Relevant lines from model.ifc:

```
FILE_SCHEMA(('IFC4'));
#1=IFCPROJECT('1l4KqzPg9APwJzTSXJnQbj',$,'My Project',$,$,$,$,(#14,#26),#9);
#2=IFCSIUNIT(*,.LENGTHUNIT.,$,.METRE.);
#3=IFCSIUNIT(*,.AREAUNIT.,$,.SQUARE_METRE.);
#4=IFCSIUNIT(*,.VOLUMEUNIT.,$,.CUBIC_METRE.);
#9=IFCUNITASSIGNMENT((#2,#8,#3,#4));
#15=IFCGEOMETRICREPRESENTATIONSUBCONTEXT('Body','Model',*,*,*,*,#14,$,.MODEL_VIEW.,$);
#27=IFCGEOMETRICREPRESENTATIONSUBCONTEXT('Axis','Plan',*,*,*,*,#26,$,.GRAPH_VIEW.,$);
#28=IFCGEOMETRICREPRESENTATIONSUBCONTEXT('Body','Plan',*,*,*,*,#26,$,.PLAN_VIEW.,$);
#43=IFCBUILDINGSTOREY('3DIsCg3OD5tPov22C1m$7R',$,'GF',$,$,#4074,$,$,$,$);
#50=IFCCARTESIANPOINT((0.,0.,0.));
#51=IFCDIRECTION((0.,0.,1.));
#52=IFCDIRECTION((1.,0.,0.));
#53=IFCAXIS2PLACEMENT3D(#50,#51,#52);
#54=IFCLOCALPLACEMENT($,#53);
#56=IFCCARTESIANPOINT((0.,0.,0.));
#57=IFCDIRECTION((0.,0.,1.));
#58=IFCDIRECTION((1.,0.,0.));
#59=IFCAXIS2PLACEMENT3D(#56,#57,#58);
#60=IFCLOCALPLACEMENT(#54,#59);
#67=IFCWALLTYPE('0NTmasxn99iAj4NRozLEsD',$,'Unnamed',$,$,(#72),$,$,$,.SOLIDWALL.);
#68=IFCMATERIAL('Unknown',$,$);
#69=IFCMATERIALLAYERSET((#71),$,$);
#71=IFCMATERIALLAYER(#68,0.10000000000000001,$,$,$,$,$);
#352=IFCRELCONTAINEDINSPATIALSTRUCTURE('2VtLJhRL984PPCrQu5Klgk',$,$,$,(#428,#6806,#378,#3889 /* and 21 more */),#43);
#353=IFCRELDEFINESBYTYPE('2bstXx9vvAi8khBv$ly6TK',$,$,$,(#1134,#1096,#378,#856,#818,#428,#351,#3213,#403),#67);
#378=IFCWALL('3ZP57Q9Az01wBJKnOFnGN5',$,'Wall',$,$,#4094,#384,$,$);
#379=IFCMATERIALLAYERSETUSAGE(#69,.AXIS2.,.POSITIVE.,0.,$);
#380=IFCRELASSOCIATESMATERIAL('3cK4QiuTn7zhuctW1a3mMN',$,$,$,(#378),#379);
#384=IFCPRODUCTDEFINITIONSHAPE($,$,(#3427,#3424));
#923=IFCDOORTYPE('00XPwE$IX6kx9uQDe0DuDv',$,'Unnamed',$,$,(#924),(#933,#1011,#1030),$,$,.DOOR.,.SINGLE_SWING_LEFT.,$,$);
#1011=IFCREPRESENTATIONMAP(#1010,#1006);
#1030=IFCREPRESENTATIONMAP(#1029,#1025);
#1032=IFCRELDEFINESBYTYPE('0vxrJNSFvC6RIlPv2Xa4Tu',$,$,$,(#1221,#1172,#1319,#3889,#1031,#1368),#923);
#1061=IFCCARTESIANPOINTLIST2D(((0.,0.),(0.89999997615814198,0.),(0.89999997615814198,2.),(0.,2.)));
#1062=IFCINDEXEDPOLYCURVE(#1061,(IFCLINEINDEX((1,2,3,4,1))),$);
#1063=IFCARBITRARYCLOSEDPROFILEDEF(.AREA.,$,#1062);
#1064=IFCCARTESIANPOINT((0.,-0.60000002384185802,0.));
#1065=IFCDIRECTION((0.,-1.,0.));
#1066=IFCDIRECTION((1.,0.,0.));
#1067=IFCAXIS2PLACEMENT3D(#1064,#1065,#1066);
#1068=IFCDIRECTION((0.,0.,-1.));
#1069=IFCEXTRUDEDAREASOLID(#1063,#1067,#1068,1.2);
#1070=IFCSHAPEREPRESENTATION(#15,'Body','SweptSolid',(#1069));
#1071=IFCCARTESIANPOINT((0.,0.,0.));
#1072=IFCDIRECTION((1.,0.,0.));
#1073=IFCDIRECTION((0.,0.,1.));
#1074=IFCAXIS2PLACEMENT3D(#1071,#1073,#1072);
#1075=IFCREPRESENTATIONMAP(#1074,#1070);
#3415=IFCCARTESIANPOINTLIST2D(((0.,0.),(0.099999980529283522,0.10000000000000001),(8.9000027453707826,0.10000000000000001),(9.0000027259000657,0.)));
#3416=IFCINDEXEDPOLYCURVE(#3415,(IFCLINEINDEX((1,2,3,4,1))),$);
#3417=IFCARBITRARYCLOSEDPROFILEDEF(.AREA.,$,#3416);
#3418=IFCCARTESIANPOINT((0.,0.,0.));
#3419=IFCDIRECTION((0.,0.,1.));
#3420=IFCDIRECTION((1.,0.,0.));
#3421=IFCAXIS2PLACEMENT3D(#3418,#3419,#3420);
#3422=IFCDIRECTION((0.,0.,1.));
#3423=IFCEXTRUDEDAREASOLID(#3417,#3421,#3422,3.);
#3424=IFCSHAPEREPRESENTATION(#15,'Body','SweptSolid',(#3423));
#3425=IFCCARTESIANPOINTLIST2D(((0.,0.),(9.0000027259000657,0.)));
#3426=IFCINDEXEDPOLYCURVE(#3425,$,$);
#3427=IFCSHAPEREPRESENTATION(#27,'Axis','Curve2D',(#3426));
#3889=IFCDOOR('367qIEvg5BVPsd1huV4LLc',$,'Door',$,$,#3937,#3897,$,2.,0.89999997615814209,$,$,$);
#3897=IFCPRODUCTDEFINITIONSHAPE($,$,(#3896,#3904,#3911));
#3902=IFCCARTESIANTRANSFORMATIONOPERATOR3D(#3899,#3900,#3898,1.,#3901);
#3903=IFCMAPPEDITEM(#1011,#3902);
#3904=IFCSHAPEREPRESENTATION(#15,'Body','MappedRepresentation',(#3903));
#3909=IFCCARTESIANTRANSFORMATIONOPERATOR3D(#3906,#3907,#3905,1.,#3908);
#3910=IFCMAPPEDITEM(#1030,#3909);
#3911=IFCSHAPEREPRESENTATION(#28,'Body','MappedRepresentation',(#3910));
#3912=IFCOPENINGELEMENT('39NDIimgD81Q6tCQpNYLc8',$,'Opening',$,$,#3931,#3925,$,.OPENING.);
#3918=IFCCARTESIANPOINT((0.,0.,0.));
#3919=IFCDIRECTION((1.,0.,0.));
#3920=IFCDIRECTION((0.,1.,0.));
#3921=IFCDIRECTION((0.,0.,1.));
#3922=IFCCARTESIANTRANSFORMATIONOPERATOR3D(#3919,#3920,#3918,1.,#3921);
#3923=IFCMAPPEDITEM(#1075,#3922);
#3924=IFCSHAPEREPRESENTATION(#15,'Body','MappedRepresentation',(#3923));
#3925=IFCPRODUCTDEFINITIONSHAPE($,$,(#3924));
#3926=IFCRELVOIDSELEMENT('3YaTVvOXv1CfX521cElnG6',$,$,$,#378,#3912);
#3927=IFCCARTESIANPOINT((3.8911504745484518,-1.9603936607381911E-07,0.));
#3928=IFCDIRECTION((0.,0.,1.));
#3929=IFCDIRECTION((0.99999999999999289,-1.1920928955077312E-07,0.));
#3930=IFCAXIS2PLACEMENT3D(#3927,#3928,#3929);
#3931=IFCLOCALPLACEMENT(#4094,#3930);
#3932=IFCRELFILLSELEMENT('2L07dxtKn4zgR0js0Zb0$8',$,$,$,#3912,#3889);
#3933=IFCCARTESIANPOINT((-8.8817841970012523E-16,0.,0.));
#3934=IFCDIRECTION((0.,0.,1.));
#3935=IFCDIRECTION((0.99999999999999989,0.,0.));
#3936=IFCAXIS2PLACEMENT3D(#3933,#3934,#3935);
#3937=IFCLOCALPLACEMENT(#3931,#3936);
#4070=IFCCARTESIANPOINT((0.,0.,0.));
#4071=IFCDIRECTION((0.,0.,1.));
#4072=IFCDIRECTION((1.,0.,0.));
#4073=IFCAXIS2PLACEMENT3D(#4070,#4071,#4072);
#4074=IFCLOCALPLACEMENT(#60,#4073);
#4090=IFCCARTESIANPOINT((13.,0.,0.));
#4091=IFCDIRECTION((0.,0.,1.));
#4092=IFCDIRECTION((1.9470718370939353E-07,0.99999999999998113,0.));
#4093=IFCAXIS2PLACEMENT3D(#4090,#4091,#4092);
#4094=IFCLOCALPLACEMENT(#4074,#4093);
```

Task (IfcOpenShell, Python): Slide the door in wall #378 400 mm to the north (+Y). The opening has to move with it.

```python
import ifcopenshell
import ifcopenshell.api.geometry
import ifcopenshell.util.placement
import ifcopenshell.util.unit

model = ifcopenshell.open("model.ifc")
unit_scale = ifcopenshell.util.unit.calculate_unit_scale(model)

door = model.by_guid("367qIEvg5BVPsd1huV4LLc")
opening = door.FillsVoids[0].RelatingOpeningElement
wall = opening.VoidsElements[0].RelatingBuildingElement

wall_matrix = ifcopenshell.util.placement.get_local_placement(wall.ObjectPlacement)
shift = wall_matrix[:3, 0] * 0.4 / unit_scale
before = ifcopenshell.util.placement.get_local_placement(door.ObjectPlacement)[:3, 3].copy()

# The door is placed relative to its opening, so it follows when the opening moves.
matrix = ifcopenshell.util.placement.get_local_placement(opening.ObjectPlacement)
matrix[:3, 3] += shift
ifcopenshell.api.geometry.edit_object_placement(
    model, product=opening, matrix=matrix, is_si=False, should_transform_children=True
)

after = ifcopenshell.util.placement.get_local_placement(door.ObjectPlacement)[:3, 3]
print("door moved by", (after - before).round(3) + 0.0)

model.write("model-out.ifc")
```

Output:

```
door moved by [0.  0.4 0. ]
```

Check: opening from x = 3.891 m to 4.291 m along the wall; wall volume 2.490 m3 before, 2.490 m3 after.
